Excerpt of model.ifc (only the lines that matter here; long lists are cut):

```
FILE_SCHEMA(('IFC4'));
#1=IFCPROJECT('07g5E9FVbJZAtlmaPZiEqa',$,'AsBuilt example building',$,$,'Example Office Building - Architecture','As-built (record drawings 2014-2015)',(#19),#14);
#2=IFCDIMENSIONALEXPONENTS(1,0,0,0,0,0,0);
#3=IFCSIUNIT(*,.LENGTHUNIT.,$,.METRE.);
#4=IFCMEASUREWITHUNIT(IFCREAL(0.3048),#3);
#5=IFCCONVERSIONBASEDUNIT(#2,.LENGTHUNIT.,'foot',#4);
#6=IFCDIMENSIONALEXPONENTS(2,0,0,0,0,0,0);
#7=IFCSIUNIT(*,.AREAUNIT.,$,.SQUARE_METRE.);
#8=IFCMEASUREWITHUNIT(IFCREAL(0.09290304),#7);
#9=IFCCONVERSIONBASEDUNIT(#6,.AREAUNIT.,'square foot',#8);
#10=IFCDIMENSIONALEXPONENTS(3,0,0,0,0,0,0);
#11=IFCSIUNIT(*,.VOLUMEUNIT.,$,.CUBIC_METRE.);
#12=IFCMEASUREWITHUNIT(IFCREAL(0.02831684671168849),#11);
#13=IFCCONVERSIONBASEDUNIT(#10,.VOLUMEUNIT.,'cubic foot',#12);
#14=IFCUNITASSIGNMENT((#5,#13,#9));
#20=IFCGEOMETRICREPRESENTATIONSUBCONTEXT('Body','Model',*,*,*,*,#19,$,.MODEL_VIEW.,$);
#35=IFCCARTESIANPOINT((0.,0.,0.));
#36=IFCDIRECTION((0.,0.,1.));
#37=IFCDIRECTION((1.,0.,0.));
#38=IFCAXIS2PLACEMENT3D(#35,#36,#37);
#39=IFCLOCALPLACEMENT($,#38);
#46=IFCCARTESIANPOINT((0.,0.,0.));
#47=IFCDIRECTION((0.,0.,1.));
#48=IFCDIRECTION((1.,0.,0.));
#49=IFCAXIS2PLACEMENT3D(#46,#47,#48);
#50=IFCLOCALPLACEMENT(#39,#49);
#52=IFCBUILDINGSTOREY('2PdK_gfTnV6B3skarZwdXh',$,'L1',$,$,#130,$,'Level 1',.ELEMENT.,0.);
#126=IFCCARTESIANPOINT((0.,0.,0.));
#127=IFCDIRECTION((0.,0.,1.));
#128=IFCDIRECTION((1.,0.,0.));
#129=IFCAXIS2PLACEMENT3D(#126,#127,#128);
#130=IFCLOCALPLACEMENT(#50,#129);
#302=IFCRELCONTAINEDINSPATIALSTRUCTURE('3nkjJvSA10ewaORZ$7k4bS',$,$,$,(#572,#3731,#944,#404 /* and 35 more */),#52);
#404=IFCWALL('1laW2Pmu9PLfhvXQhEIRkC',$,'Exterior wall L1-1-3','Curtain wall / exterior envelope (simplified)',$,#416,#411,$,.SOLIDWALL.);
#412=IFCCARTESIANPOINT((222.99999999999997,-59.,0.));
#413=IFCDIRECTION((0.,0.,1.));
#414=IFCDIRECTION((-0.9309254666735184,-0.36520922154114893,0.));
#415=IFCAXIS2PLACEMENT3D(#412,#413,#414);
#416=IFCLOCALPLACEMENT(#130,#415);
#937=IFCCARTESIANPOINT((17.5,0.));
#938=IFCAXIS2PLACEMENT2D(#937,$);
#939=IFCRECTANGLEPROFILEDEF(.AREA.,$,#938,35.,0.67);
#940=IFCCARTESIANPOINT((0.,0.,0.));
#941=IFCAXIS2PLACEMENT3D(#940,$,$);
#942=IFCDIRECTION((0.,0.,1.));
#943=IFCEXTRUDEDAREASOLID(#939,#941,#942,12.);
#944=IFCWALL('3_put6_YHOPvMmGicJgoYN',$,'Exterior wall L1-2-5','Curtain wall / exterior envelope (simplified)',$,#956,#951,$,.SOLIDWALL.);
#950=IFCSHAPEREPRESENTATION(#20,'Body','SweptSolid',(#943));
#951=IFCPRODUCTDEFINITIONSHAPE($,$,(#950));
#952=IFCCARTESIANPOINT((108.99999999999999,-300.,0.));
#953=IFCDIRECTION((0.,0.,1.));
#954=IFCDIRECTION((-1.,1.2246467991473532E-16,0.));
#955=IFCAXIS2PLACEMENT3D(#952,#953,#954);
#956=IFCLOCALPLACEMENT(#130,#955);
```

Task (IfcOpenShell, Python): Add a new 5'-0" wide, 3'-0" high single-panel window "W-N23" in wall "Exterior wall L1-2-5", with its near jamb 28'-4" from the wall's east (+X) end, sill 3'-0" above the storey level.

```python
import numpy as np
import ifcopenshell
import ifcopenshell.api.feature
import ifcopenshell.api.geometry
import ifcopenshell.api.root
import ifcopenshell.api.spatial
import ifcopenshell.geom
import ifcopenshell.util.element
import ifcopenshell.util.placement
import ifcopenshell.util.representation
import ifcopenshell.util.shape
import ifcopenshell.util.unit

model = ifcopenshell.open("model.ifc")
unit_scale = ifcopenshell.util.unit.calculate_unit_scale(model)
settings = ifcopenshell.geom.settings()


def volume(element):
    """Net volume in cubic metres, openings subtracted."""
    shape = ifcopenshell.geom.create_shape(settings, element)
    return ifcopenshell.util.shape.get_volume(shape.geometry)


wall = model.by_id(944)
storey = ifcopenshell.util.element.get_container(wall, ifc_class="IfcBuildingStorey")
context = ifcopenshell.util.representation.get_context(model, "Model", "Body", "MODEL_VIEW")
before = volume(wall)

width, height, from_end, sill = 1.524, 0.9144, 8.636, 0.9144  # metres

# The wall runs along its own X axis, and the end named is its -X end.
wall_shape = ifcopenshell.geom.create_shape(settings, wall)
x, y, z = ifcopenshell.util.shape.get_vertices(wall_shape.geometry).T
start = x.min() + from_end
face, thickness = float(y.min()), float(y.max() - y.min())
wall_matrix = ifcopenshell.util.placement.get_local_placement(wall.ObjectPlacement)
level = ifcopenshell.util.placement.get_local_placement(storey.ObjectPlacement)[2, 3]


def in_wall(x, y):
    """Placement at x, y metres in the wall's axes, at sill height."""
    matrix = wall_matrix.copy()
    matrix[:, 3] = wall_matrix @ np.array([x / unit_scale, y / unit_scale, 0.0, 1.0])
    matrix[2, 3] = level + sill / unit_scale
    return matrix


# Opening: a box that overshoots both wall faces by 50 mm.
opening = ifcopenshell.api.root.create_entity(model, ifc_class="IfcOpeningElement", predefined_type="OPENING")
box = ifcopenshell.api.geometry.add_wall_representation(
    model, context=context, length=width, height=height, thickness=thickness + 0.1
)
ifcopenshell.api.geometry.assign_representation(model, product=opening, representation=box)
ifcopenshell.api.geometry.edit_object_placement(model, product=opening, matrix=in_wall(start, face - 0.05), is_si=False)
ifcopenshell.api.feature.add_feature(model, feature=opening, element=wall)

window = ifcopenshell.api.root.create_entity(model, ifc_class="IfcWindow", name="W-N23", predefined_type="WINDOW")
window.OverallWidth, window.OverallHeight = width / unit_scale, height / unit_scale
window.PartitioningType = "SINGLE_PANEL"
body = ifcopenshell.api.geometry.add_window_representation(
    model,
    context=context,
    overall_width=window.OverallWidth,
    overall_height=window.OverallHeight,
    partition_type="SINGLE_PANEL",
)
ifcopenshell.api.geometry.assign_representation(model, product=window, representation=body)
ifcopenshell.api.spatial.assign_container(model, products=[window], relating_structure=storey)
ifcopenshell.api.feature.add_filling(model, opening=opening, element=window)

# Centre the window in the wall's thickness.
ifcopenshell.api.geometry.edit_object_placement(model, product=window, matrix=in_wall(start, face), is_si=False)
window_shape = ifcopenshell.geom.create_shape(settings, window)
depth = ifcopenshell.util.shape.get_vertices(window_shape.geometry)[:, 1]
offset = face + thickness / 2 - (depth.min() + depth.max()) / 2
ifcopenshell.api.geometry.edit_object_placement(model, product=window, matrix=in_wall(start, offset), is_si=False)

after = volume(wall)

print(f"wall volume {before:.3f} -> {after:.3f} m3")

model.write("model_updated.ifc")
```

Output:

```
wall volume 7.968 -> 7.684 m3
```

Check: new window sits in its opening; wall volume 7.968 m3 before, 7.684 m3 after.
